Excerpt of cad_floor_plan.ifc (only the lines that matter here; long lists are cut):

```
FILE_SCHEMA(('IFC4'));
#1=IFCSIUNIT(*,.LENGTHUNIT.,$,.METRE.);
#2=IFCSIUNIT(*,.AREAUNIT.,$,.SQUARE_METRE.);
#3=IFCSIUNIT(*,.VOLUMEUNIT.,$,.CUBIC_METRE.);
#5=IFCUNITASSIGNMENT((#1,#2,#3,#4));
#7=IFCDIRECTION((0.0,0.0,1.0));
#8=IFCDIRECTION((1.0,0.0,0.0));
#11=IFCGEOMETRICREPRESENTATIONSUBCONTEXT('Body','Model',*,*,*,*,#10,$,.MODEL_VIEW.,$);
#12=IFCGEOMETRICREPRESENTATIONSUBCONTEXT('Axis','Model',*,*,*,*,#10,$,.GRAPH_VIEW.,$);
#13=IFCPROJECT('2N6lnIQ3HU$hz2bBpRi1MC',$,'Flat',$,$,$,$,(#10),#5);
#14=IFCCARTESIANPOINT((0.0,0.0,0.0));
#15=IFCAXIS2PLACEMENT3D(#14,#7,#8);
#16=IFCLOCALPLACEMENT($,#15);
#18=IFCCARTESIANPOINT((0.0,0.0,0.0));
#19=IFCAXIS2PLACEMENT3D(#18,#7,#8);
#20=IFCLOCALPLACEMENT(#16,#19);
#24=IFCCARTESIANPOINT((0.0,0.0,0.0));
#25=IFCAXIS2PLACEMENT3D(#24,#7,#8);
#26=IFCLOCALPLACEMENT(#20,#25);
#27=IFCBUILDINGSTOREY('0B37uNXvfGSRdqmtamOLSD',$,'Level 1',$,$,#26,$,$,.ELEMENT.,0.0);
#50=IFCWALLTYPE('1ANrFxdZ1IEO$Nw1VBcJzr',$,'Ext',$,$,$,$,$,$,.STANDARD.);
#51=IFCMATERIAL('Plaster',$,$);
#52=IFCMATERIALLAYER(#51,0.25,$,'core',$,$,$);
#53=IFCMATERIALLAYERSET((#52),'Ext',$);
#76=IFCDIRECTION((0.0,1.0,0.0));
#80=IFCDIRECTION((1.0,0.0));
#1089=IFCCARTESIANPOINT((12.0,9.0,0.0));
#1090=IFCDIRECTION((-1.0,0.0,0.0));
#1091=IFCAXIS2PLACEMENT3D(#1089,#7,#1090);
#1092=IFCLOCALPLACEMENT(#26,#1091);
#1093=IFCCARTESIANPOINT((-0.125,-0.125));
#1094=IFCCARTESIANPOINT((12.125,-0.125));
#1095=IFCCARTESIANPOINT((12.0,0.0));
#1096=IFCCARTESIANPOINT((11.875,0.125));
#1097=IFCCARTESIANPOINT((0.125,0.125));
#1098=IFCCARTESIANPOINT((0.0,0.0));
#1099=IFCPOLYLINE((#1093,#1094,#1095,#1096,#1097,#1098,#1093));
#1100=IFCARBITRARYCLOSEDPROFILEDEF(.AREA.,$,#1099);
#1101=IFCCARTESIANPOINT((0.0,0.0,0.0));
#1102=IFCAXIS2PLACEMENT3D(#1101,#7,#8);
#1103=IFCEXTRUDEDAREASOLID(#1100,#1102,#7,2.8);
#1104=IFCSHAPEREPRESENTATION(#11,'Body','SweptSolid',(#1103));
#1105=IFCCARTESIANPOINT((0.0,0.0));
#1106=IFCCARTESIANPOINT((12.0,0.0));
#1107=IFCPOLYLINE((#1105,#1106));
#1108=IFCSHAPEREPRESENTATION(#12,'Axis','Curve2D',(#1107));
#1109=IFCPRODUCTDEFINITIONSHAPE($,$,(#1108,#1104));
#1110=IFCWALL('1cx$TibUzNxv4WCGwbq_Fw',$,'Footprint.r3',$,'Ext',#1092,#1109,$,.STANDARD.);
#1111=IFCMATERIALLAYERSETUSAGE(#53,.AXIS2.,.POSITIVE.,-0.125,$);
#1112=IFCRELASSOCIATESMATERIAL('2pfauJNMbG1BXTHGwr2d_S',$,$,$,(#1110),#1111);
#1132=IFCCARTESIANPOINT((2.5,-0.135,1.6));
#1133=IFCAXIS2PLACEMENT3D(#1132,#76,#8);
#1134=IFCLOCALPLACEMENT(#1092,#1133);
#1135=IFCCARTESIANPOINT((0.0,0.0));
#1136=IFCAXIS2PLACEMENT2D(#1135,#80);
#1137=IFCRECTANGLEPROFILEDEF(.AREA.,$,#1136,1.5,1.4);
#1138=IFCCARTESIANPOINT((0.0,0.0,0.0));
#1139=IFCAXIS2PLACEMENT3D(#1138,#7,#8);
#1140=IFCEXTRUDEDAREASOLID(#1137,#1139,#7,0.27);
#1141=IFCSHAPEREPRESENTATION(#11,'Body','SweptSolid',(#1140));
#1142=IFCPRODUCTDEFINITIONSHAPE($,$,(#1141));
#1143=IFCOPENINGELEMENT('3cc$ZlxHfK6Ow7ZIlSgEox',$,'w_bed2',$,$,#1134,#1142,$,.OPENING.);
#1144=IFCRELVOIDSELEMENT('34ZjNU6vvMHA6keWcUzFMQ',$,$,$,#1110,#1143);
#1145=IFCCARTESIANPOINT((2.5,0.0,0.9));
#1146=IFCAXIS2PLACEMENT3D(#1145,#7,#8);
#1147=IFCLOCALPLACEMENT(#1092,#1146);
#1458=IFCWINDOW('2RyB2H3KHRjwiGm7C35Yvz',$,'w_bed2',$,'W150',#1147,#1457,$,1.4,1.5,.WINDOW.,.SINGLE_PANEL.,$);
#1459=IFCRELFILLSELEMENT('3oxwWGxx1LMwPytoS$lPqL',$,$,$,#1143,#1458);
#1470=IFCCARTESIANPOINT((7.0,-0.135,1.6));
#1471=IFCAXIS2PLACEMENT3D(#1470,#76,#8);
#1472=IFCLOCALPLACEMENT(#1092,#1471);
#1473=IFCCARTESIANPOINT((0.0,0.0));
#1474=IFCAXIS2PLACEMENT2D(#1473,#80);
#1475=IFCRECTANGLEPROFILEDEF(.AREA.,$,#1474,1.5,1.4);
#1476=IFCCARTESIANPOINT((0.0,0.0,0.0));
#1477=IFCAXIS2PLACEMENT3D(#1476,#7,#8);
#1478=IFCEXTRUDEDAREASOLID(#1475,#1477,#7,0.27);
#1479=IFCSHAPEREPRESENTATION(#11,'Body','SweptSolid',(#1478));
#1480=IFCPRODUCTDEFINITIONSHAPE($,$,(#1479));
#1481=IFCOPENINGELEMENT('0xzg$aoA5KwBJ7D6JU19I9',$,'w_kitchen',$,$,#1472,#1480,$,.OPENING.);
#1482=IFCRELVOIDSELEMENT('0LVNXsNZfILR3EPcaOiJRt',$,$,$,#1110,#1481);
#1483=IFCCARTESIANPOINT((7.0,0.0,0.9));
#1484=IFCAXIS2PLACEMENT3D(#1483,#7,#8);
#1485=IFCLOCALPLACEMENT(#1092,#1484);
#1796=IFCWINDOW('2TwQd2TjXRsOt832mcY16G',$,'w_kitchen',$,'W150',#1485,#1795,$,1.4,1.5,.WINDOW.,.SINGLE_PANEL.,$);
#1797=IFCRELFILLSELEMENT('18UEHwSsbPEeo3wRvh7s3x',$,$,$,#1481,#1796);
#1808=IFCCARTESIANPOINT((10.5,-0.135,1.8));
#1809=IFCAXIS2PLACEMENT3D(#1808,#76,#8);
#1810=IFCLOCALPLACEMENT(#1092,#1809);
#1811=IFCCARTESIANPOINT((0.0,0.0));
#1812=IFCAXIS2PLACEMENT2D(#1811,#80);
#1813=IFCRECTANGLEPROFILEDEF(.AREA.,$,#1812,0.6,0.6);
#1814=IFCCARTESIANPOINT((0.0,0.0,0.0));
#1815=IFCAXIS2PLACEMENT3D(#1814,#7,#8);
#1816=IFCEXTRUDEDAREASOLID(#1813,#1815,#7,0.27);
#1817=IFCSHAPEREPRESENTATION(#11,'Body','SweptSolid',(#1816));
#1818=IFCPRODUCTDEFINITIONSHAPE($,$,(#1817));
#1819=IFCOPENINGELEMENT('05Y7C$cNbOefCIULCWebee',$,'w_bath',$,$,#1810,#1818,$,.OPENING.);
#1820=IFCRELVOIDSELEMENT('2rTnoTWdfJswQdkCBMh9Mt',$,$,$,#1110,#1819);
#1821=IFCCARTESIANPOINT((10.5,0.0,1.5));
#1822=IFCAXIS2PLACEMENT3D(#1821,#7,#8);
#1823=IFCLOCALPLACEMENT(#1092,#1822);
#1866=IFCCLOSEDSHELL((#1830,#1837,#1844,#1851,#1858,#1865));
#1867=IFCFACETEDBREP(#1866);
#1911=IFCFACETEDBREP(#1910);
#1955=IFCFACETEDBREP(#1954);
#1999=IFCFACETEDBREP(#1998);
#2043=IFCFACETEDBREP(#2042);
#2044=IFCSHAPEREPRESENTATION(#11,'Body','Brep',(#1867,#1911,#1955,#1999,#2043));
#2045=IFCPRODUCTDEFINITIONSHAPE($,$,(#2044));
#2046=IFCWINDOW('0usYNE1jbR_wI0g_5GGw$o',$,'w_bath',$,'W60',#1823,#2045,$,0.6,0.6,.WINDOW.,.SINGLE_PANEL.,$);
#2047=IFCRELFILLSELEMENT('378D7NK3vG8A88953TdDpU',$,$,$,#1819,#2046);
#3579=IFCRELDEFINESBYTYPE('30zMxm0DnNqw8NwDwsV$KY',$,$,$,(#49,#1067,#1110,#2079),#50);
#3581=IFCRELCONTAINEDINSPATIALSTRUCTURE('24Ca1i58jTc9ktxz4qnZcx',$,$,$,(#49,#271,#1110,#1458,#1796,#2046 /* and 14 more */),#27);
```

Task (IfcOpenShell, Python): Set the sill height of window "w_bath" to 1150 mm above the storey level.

```python
import numpy as np
import ifcopenshell
import ifcopenshell.api.geometry
import ifcopenshell.geom
import ifcopenshell.util.element
import ifcopenshell.util.placement
import ifcopenshell.util.shape
import ifcopenshell.util.unit

model = ifcopenshell.open("cad_floor_plan.ifc")
unit_scale = ifcopenshell.util.unit.calculate_unit_scale(model)

window = model.by_guid("0usYNE1jbR_wI0g_5GGw$o")
opening = window.FillsVoids[0].RelatingOpeningElement
storey = ifcopenshell.util.element.get_container(window, ifc_class="IfcBuildingStorey")
level = ifcopenshell.util.placement.get_local_placement(storey.ObjectPlacement)[2, 3]

# The opening's origin need not be at the sill, so measure its lowest point.
shape = ifcopenshell.geom.create_shape(ifcopenshell.geom.settings(), opening)
bottom = ifcopenshell.util.shape.get_shape_bottom_elevation(shape, shape.geometry) / unit_scale
dz = level + 1.15 - bottom

shift = np.array([0.0, 0.0, dz])
# The window is not placed relative to its opening, so move both.
for product in (opening, window):
    matrix = ifcopenshell.util.placement.get_local_placement(product.ObjectPlacement)
    matrix[:3, 3] += shift
    ifcopenshell.api.geometry.edit_object_placement(model, product=product, matrix=matrix, is_si=False)

print(f"moved by {dz * unit_scale:+.3f} m")

model.write("cad_floor_plan_v2.ifc")
```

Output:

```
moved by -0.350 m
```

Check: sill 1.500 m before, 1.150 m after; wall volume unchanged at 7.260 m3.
